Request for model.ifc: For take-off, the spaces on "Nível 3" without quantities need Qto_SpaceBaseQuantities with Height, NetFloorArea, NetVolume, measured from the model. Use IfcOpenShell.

First a look at what the model holds.

```python
import ifcopenshell
import ifcopenshell.util.element
import ifcopenshell.util.unit

model = ifcopenshell.open("model.ifc")
print(model.schema)
for unit_type in ("LENGTHUNIT", "AREAUNIT", "VOLUMEUNIT"):
    print(unit_type, ifcopenshell.util.unit.calculate_unit_scale(model, unit_type))
storey = next(s for s in model.by_type("IfcBuildingStorey") if s.Name == "Nível 3")
spaces = [e for e in ifcopenshell.util.element.get_decomposition(storey) if e.is_a("IfcSpace")]
for e in sorted(spaces, key=lambda e: e.id()):
    print(e.id(), e.is_a(), e.Name, list(ifcopenshell.util.element.get_psets(e, qtos_only=True)), sep=" | ")
```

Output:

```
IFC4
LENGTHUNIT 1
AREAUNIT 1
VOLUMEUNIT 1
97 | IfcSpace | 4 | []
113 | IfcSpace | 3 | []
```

```python
import ifcopenshell
import ifcopenshell.api.pset
import ifcopenshell.geom
import ifcopenshell.util.element
import ifcopenshell.util.shape
import ifcopenshell.util.unit

model = ifcopenshell.open("model.ifc")
unit_scale = ifcopenshell.util.unit.calculate_unit_scale(model)
area_scale = ifcopenshell.util.unit.calculate_unit_scale(model, "AREAUNIT")
volume_scale = ifcopenshell.util.unit.calculate_unit_scale(model, "VOLUMEUNIT")
settings = ifcopenshell.geom.settings()

storey = next(s for s in model.by_type("IfcBuildingStorey") if s.Name == "Nível 3")
spaces = [e for e in ifcopenshell.util.element.get_decomposition(storey) if e.is_a("IfcSpace")]

for e in sorted(spaces, key=lambda e: e.id()):
    if ifcopenshell.util.element.get_psets(e, qtos_only=True, should_inherit=False):
        continue
    # Geometry comes back in metres, in the element's own axes.
    shape = ifcopenshell.geom.create_shape(settings, e)
    values = {
        "Height": ifcopenshell.util.shape.get_z(shape.geometry) / unit_scale,
        "NetFloorArea": ifcopenshell.util.shape.get_footprint_area(shape.geometry) / area_scale,
        "NetVolume": ifcopenshell.util.shape.get_volume(shape.geometry) / volume_scale,
    }
    qto = ifcopenshell.api.pset.add_qto(model, product=e, name="Qto_SpaceBaseQuantities")
    ifcopenshell.api.pset.edit_qto(model, qto=qto, properties=values)
    print(e.id(), {k: round(v, 3) for k, v in values.items()})

model.write("model_updated.ifc")
```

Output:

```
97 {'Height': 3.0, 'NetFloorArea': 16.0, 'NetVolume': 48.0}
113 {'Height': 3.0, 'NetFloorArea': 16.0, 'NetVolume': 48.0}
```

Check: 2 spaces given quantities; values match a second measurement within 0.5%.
